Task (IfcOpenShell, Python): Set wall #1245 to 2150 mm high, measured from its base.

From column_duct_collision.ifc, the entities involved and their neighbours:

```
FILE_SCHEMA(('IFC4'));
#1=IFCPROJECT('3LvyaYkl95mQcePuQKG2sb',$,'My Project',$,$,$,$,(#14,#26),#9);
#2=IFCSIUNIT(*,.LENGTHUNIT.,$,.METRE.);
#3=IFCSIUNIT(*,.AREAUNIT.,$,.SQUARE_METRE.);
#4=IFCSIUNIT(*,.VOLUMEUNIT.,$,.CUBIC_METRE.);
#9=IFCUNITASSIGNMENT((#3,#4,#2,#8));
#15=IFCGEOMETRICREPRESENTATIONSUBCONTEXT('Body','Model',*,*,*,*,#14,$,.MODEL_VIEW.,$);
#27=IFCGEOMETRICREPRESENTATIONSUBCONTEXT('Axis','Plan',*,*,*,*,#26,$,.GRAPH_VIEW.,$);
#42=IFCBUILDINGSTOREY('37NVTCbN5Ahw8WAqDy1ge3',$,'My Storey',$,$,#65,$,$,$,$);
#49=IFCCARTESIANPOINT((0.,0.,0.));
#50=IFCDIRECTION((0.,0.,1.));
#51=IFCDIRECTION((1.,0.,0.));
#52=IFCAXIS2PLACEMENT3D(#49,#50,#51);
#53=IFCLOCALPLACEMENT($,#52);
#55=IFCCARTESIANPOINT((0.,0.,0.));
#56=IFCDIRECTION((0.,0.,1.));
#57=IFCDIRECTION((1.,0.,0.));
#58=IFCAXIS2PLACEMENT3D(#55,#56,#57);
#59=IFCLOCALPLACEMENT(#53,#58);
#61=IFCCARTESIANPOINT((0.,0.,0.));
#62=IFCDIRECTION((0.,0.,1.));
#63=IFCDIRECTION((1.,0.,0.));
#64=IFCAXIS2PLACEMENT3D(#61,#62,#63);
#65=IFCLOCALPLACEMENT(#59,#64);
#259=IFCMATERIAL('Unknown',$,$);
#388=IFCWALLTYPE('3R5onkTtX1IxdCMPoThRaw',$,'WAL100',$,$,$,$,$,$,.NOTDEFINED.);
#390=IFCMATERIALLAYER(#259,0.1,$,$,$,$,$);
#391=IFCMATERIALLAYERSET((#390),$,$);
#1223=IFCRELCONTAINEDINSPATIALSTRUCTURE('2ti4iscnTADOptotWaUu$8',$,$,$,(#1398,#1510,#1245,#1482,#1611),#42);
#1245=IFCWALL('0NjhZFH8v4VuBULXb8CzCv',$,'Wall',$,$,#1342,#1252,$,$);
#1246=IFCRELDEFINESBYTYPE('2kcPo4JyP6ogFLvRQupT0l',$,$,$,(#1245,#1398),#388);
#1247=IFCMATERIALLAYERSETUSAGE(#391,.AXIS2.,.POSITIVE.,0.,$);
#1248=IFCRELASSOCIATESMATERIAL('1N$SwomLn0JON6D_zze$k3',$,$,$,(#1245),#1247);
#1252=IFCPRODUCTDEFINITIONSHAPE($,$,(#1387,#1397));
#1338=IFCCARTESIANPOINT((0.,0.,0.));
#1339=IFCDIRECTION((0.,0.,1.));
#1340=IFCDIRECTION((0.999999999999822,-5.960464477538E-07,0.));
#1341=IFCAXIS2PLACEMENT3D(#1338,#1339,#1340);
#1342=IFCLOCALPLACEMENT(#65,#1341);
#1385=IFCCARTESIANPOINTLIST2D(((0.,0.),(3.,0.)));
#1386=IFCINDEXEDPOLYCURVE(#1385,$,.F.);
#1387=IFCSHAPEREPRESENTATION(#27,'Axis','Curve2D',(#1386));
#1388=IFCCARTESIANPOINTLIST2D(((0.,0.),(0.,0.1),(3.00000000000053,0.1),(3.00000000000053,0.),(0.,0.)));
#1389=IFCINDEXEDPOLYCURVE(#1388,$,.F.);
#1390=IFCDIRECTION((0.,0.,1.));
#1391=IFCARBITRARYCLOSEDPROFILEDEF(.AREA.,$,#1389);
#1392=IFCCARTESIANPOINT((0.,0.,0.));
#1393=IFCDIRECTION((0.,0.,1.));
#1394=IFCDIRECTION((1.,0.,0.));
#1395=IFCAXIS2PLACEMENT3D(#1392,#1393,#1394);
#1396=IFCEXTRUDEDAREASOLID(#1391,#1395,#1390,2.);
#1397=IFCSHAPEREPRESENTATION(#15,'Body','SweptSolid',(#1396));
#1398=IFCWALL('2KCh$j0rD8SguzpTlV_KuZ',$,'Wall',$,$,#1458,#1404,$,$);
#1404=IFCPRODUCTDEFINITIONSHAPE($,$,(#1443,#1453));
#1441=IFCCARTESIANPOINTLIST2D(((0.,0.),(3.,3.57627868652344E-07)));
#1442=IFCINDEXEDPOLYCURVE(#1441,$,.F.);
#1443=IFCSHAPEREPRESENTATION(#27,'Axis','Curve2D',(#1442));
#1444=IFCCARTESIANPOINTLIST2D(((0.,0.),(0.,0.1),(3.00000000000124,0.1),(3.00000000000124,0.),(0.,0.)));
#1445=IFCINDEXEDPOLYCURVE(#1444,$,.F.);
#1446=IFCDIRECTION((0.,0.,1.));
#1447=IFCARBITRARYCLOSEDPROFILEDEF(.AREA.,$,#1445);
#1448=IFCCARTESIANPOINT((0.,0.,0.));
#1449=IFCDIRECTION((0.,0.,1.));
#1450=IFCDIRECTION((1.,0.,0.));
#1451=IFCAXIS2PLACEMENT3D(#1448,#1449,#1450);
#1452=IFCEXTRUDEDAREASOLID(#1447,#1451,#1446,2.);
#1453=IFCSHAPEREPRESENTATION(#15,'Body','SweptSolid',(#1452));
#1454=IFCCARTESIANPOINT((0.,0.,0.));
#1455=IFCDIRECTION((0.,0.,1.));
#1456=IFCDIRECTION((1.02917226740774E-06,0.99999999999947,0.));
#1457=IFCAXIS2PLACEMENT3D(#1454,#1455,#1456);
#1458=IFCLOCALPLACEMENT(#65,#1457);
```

```python
import ifcopenshell
import ifcopenshell.geom
import ifcopenshell.util.representation
import ifcopenshell.util.shape
import ifcopenshell.util.unit

model = ifcopenshell.open("column_duct_collision.ifc")
unit_scale = ifcopenshell.util.unit.calculate_unit_scale(model)
settings = ifcopenshell.geom.settings()


def volume(element):
    """Net volume in cubic metres, openings subtracted."""
    shape = ifcopenshell.geom.create_shape(settings, element)
    return ifcopenshell.util.shape.get_volume(shape.geometry)


wall = model.by_guid("0NjhZFH8v4VuBULXb8CzCv")
before = volume(wall)

body = ifcopenshell.util.representation.get_representation(wall, "Model", "Body")
solid = body.Items[0]
old_height = solid.Depth
solid.Depth = 2.15 / unit_scale
after = volume(wall)

print(f"height {old_height:g} -> {solid.Depth:g}, volume {before:.3f} -> {after:.3f} m3")

model.write("column_duct_collision_edited.ifc")
```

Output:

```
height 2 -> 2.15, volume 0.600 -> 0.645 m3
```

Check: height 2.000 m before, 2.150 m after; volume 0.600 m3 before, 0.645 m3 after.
